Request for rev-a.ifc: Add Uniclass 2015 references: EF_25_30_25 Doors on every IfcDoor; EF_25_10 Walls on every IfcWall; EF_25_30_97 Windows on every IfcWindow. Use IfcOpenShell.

First a look at what the model holds.

```python
import ifcopenshell

model = ifcopenshell.open("rev-a.ifc")
print(model.schema)
print("classifications:", [c.Name for c in model.by_type("IfcClassification")])
for ifc_class in ("IfcDoor", "IfcRoof", "IfcStair", "IfcWall", "IfcWindow"):
    print(ifc_class, len(model.by_type(ifc_class)))
```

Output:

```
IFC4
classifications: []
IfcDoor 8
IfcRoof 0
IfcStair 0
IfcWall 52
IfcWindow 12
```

```python
import ifcopenshell
import ifcopenshell.api.classification

model = ifcopenshell.open("rev-a.ifc")

system = ifcopenshell.api.classification.add_classification(model, classification="Uniclass 2015")

codes = {
    "IfcDoor": ("EF_25_30_25", "Doors"),
    "IfcWall": ("EF_25_10", "Walls"),
    "IfcWindow": ("EF_25_30_97", "Windows"),
}
for ifc_class, (code, name) in codes.items():
    products = model.by_type(ifc_class)
    ifcopenshell.api.classification.add_reference(
        model, products=products, classification=system, identification=code, name=name
    )
    print(code, len(products))

model.write("rev-a-out.ifc")
```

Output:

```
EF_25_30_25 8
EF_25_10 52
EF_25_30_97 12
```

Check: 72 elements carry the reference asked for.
